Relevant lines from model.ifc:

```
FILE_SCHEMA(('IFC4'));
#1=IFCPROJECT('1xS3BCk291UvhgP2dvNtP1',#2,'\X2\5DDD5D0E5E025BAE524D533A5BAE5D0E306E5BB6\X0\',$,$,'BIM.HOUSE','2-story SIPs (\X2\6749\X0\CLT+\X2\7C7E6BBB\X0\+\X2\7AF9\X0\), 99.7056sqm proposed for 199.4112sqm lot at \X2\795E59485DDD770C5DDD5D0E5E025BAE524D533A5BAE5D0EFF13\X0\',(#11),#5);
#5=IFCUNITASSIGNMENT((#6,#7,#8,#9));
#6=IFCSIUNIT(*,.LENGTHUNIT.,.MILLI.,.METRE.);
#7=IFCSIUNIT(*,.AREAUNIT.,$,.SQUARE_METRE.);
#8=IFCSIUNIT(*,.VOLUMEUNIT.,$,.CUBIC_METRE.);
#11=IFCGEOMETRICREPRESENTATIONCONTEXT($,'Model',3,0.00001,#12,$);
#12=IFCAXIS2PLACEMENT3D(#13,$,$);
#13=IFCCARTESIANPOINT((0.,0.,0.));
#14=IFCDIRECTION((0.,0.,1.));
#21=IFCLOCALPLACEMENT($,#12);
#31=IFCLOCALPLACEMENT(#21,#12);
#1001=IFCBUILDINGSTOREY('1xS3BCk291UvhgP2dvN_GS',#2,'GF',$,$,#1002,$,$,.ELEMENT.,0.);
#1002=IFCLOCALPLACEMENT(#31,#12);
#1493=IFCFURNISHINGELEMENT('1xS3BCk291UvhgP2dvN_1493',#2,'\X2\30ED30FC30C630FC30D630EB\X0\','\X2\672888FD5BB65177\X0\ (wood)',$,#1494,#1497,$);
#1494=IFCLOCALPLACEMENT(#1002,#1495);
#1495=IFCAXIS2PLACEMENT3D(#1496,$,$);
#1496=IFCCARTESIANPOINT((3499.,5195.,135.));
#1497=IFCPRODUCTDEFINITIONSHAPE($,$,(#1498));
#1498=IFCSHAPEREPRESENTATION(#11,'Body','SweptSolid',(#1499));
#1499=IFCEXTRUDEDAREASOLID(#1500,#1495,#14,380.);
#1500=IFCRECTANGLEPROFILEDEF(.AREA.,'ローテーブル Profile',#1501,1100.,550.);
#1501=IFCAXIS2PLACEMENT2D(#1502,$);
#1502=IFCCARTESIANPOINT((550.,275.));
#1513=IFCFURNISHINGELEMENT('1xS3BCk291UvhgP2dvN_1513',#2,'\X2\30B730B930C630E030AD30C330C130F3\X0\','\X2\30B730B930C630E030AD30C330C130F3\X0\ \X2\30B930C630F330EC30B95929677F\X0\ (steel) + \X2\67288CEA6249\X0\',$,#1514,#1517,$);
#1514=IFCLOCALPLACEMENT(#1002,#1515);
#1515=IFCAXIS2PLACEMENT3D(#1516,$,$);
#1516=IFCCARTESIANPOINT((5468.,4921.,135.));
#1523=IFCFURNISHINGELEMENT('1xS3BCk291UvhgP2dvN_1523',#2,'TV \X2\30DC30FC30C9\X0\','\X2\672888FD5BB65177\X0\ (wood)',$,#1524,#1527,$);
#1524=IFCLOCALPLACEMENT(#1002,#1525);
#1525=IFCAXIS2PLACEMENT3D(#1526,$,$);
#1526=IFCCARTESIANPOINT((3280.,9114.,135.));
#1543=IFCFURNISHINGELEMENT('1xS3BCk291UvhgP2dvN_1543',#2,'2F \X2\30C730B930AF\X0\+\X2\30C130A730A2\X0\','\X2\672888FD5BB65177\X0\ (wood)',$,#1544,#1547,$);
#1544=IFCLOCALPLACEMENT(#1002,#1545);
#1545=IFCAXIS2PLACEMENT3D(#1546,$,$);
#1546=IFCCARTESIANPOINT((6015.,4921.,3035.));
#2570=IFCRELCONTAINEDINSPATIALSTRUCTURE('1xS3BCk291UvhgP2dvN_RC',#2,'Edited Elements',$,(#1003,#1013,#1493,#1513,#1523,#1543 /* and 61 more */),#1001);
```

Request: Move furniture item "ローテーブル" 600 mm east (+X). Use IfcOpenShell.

```python
import ifcopenshell
import ifcopenshell.api.geometry
import ifcopenshell.util.placement

model = ifcopenshell.open("model.ifc")

item = model.by_id(1493)
matrix = ifcopenshell.util.placement.get_local_placement(item.ObjectPlacement)
matrix[0, 3] += 600.0
ifcopenshell.api.geometry.edit_object_placement(model, product=item, matrix=matrix, is_si=False)

print(ifcopenshell.util.placement.get_local_placement(item.ObjectPlacement).round(3) + 0.0)

model.write("model_rev.ifc")
```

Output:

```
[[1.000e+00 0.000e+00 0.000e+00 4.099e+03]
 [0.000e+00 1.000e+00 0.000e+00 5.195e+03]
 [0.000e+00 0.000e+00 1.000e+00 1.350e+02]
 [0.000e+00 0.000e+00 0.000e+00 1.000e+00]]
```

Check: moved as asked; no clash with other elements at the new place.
